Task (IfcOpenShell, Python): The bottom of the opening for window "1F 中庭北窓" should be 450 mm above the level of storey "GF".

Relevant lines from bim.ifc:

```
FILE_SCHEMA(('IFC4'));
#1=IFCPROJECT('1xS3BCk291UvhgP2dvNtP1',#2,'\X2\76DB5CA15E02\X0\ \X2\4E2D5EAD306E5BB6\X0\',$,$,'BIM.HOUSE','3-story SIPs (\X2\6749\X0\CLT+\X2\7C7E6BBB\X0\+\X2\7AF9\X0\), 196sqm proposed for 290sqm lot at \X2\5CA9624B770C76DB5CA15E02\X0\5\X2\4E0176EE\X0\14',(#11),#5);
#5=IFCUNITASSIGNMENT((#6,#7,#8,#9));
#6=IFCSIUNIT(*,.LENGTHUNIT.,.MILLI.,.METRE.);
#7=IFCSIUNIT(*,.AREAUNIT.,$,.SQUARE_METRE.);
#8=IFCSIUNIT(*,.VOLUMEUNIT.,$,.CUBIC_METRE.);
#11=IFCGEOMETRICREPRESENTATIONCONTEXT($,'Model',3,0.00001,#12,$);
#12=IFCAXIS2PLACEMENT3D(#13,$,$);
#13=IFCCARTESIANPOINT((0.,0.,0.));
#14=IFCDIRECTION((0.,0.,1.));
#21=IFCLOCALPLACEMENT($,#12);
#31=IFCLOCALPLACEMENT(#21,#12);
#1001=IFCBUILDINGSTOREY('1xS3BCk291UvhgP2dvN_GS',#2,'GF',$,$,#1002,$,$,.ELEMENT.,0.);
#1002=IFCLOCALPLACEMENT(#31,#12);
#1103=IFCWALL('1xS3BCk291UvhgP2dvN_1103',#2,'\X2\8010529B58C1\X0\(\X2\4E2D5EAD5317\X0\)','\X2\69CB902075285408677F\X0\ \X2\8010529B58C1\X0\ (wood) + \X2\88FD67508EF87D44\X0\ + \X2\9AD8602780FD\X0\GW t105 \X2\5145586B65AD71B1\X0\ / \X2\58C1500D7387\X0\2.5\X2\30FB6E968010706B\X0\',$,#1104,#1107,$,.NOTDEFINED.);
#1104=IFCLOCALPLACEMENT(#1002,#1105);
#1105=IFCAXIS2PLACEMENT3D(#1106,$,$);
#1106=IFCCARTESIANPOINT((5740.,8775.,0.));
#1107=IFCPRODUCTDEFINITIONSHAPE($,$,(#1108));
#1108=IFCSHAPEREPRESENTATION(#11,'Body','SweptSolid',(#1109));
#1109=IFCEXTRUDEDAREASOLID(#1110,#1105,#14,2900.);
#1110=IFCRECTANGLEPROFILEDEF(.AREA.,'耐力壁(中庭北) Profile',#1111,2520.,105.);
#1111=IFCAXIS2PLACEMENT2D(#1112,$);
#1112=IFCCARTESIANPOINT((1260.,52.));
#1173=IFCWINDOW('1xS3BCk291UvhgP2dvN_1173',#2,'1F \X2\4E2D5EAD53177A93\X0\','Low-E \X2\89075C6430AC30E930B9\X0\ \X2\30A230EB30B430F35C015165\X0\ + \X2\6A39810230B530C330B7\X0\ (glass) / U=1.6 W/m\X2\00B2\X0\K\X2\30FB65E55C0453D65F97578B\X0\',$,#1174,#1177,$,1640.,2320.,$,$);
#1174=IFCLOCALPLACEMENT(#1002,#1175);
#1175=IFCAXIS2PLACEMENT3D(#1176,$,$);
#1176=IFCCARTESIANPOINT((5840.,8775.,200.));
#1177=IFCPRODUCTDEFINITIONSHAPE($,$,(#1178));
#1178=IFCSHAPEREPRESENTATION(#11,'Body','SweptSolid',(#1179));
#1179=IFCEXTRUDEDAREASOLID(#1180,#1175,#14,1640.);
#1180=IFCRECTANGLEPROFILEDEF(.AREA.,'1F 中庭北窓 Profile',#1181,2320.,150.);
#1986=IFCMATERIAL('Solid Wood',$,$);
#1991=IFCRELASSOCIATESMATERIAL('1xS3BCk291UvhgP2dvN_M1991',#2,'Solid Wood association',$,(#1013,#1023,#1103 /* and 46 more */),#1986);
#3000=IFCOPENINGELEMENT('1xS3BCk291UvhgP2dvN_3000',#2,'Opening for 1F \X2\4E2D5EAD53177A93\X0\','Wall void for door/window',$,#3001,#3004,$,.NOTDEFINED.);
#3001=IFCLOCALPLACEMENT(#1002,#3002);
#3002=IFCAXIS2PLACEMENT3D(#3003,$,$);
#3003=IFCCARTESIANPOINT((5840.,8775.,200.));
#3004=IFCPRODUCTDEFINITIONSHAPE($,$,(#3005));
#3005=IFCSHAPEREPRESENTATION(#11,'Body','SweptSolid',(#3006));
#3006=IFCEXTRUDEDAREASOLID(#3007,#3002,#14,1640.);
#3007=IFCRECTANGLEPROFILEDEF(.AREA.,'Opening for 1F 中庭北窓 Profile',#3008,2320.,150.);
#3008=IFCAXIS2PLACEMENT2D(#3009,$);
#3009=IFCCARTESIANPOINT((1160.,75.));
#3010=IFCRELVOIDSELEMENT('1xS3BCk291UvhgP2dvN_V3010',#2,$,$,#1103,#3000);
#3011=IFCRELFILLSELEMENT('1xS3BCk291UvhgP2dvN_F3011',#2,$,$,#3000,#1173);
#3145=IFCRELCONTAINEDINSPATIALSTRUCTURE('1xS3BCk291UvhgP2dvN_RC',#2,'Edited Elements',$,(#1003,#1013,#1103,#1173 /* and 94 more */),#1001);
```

```python
import numpy as np
import ifcopenshell
import ifcopenshell.api.geometry
import ifcopenshell.geom
import ifcopenshell.util.element
import ifcopenshell.util.placement
import ifcopenshell.util.shape
import ifcopenshell.util.unit

model = ifcopenshell.open("bim.ifc")
unit_scale = ifcopenshell.util.unit.calculate_unit_scale(model)

window = model.by_guid("1xS3BCk291UvhgP2dvN_1173")
opening = window.FillsVoids[0].RelatingOpeningElement
storey = ifcopenshell.util.element.get_container(window, ifc_class="IfcBuildingStorey")
level = ifcopenshell.util.placement.get_local_placement(storey.ObjectPlacement)[2, 3]

# The opening's origin need not be at the sill, so measure its lowest point.
shape = ifcopenshell.geom.create_shape(ifcopenshell.geom.settings(), opening)
bottom = ifcopenshell.util.shape.get_shape_bottom_elevation(shape, shape.geometry) / unit_scale
dz = level + 0.45 / unit_scale - bottom

shift = np.array([0.0, 0.0, dz])
# The window is not placed relative to its opening, so move both.
for product in (opening, window):
    matrix = ifcopenshell.util.placement.get_local_placement(product.ObjectPlacement)
    matrix[:3, 3] += shift
    ifcopenshell.api.geometry.edit_object_placement(model, product=product, matrix=matrix, is_si=False)

print(f"moved by {dz * unit_scale:+.3f} m")

model.write("bim_edited.ifc")
```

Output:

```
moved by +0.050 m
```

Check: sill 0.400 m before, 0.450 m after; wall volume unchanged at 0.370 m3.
